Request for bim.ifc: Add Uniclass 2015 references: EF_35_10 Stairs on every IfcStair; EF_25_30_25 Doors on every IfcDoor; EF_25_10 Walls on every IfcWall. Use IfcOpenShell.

First a look at what the model holds.

```python
import ifcopenshell

model = ifcopenshell.open("bim.ifc")
print(model.schema)
print("classifications:", [c.Name for c in model.by_type("IfcClassification")])
for ifc_class in ("IfcDoor", "IfcRoof", "IfcStair", "IfcWall", "IfcWindow"):
    print(ifc_class, len(model.by_type(ifc_class)))
```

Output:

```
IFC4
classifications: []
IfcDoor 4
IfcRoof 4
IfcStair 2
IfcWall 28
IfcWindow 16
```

```python
import ifcopenshell
import ifcopenshell.api.classification

model = ifcopenshell.open("bim.ifc")

system = ifcopenshell.api.classification.add_classification(model, classification="Uniclass 2015")

codes = {
    "IfcStair": ("EF_35_10", "Stairs"),
    "IfcDoor": ("EF_25_30_25", "Doors"),
    "IfcWall": ("EF_25_10", "Walls"),
}
for ifc_class, (code, name) in codes.items():
    products = model.by_type(ifc_class)
    ifcopenshell.api.classification.add_reference(
        model, products=products, classification=system, identification=code, name=name
    )
    print(code, len(products))

model.write("bim_updated.ifc")
```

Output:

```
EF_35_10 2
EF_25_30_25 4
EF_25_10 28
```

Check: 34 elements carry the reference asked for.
